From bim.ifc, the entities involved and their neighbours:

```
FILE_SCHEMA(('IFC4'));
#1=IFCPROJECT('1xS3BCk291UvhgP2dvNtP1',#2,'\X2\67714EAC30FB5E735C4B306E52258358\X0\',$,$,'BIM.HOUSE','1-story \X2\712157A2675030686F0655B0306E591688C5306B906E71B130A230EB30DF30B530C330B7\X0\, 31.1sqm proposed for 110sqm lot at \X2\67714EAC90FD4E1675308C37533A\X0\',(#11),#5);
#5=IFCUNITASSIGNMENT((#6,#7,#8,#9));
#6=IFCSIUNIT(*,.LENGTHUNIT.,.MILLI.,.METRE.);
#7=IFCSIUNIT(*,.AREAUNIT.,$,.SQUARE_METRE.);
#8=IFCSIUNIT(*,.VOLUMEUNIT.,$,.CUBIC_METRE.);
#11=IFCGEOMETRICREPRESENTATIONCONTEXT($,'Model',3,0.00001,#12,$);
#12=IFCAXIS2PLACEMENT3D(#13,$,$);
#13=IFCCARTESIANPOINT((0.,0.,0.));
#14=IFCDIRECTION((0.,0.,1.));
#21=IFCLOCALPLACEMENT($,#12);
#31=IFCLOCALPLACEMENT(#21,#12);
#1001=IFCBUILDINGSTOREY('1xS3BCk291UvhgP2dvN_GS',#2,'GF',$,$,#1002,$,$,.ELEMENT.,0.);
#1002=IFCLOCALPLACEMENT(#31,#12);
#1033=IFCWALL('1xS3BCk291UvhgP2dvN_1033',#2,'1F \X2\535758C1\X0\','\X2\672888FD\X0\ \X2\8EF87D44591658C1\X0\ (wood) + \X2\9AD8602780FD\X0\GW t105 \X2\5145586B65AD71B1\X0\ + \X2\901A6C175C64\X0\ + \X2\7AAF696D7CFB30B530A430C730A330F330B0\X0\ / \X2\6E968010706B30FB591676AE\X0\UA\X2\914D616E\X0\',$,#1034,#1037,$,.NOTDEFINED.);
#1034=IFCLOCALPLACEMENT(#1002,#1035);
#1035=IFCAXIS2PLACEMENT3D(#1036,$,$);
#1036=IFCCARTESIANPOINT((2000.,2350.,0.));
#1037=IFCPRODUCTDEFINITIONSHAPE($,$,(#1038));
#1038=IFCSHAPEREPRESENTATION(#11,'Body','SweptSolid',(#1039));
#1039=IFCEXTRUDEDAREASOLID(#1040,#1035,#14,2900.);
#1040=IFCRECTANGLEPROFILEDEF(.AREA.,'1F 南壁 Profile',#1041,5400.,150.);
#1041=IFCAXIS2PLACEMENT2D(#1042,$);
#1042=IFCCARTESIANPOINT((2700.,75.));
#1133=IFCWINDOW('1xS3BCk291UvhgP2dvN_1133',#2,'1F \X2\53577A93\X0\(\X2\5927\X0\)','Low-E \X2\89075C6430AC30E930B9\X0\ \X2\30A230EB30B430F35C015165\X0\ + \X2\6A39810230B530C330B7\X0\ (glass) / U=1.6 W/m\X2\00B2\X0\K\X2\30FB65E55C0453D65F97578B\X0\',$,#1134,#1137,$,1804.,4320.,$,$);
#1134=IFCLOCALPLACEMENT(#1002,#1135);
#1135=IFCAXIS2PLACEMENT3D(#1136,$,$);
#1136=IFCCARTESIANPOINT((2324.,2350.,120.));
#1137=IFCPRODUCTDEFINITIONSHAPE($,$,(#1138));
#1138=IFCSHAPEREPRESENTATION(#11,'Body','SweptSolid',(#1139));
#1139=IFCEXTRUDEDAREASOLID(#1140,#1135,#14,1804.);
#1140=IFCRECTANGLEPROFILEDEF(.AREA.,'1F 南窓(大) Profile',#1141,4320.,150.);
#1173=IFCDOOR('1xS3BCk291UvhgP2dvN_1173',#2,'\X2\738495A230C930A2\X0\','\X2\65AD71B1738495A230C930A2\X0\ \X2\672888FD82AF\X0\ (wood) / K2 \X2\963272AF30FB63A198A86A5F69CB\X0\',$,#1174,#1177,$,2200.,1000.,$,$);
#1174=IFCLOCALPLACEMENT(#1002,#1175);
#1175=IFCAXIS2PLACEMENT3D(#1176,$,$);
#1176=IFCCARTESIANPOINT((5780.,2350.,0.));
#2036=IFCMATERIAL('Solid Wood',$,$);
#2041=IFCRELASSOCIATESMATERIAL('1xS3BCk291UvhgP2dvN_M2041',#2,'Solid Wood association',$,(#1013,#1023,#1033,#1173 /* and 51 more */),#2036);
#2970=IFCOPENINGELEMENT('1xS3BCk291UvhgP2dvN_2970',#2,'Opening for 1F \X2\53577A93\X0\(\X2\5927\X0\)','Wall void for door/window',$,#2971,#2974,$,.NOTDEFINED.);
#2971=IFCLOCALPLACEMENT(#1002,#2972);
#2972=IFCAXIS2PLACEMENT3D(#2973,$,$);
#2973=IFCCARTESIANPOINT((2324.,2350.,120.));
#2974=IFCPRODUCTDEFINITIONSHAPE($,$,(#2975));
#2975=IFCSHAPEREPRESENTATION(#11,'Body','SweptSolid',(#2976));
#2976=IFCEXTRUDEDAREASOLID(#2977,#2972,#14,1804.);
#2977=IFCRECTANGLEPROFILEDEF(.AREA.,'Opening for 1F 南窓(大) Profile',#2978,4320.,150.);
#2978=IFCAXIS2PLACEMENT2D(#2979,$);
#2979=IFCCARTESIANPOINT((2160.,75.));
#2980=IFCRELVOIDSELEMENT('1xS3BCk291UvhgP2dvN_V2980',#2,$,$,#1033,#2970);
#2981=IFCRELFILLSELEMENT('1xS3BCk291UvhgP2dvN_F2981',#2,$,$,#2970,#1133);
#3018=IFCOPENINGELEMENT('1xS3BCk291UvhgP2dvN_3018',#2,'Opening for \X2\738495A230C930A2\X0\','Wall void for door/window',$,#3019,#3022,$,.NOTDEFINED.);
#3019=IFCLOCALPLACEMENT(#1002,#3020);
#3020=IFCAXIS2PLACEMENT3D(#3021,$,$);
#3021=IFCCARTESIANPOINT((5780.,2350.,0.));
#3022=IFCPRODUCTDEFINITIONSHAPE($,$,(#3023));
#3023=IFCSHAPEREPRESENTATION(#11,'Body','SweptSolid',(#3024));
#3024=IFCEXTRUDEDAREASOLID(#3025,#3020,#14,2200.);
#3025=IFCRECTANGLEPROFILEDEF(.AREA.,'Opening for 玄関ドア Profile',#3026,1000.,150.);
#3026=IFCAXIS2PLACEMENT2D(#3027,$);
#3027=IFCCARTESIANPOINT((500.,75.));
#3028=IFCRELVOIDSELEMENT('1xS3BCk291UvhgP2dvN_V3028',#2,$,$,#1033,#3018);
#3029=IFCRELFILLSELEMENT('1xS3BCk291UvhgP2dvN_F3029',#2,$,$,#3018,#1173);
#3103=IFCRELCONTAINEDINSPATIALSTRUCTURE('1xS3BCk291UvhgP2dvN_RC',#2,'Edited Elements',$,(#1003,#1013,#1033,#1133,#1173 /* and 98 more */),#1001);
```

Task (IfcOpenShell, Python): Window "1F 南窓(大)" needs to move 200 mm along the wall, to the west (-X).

```python
import ifcopenshell
import ifcopenshell.api.geometry
import ifcopenshell.util.placement

model = ifcopenshell.open("bim.ifc")

window = model.by_id(1133)
opening = window.FillsVoids[0].RelatingOpeningElement
wall = opening.VoidsElements[0].RelatingBuildingElement

wall_matrix = ifcopenshell.util.placement.get_local_placement(wall.ObjectPlacement)
shift = wall_matrix[:3, 0] * -200.0
before = ifcopenshell.util.placement.get_local_placement(window.ObjectPlacement)[:3, 3].copy()

# The window is not placed relative to its opening, so move both.
for product in (opening, window):
    matrix = ifcopenshell.util.placement.get_local_placement(product.ObjectPlacement)
    matrix[:3, 3] += shift
    ifcopenshell.api.geometry.edit_object_placement(model, product=product, matrix=matrix, is_si=False)

after = ifcopenshell.util.placement.get_local_placement(window.ObjectPlacement)[:3, 3]
print("window moved by", (after - before).round(3) + 0.0)

model.write("bim_edited.ifc")
```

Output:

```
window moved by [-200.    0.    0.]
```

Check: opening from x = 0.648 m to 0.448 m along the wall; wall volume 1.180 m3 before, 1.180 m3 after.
